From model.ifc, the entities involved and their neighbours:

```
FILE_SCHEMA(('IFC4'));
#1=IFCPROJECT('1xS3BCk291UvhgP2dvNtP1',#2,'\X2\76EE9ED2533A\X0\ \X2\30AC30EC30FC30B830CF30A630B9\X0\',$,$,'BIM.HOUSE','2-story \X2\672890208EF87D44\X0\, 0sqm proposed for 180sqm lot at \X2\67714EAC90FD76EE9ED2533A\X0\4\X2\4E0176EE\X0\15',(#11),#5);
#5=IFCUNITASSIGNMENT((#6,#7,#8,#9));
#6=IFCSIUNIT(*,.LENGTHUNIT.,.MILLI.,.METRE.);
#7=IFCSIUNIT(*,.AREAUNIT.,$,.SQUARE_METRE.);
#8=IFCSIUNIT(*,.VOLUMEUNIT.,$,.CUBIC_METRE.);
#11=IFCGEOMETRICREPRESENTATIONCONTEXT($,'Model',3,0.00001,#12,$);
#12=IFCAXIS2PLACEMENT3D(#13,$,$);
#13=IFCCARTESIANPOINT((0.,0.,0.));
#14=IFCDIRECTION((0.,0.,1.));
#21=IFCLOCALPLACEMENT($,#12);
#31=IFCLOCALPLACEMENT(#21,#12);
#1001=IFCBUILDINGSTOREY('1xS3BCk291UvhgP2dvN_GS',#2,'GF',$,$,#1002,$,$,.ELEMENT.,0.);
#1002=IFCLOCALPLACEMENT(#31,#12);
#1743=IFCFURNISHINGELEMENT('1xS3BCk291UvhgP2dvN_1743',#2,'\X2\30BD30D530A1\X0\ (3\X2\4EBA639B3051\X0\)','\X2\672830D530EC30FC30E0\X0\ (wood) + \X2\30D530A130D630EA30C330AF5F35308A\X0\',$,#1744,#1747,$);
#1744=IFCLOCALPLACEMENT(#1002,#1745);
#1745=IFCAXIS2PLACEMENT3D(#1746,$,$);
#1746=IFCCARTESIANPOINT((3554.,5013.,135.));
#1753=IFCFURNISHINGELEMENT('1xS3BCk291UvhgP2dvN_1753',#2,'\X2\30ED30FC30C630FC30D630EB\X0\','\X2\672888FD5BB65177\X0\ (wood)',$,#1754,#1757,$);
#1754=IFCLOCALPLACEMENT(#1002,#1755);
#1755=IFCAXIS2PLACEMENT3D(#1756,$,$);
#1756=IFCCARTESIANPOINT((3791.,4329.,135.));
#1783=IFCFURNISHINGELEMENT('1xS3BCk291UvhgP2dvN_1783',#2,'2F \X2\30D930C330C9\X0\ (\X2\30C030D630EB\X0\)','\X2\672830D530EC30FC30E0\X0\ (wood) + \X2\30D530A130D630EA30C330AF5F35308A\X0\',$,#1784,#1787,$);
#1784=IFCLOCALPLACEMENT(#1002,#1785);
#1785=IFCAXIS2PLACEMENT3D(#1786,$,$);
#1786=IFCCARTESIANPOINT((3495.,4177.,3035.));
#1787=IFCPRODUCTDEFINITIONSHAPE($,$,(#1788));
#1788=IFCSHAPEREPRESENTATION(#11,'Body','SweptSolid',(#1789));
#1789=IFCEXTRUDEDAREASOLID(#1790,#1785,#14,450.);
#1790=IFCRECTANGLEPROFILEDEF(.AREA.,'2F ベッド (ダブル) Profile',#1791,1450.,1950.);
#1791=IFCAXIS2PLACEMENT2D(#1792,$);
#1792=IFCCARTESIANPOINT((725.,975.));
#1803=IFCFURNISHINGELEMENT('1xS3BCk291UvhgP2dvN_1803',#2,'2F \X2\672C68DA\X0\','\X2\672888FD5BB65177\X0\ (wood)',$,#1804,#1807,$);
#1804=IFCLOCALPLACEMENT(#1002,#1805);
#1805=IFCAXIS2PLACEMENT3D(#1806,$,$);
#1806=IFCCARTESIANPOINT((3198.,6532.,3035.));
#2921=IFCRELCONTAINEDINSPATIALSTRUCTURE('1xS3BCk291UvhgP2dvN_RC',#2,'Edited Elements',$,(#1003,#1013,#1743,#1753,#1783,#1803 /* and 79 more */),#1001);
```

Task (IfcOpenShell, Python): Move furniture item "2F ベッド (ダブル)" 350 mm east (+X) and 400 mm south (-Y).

```python
import ifcopenshell
import ifcopenshell.api.geometry
import ifcopenshell.util.placement
import ifcopenshell.util.unit

model = ifcopenshell.open("model.ifc")
unit_scale = ifcopenshell.util.unit.calculate_unit_scale(model)

item = model.by_guid("1xS3BCk291UvhgP2dvN_1783")
matrix = ifcopenshell.util.placement.get_local_placement(item.ObjectPlacement)
matrix[0, 3] += 0.35 / unit_scale
matrix[1, 3] -= 0.4 / unit_scale
ifcopenshell.api.geometry.edit_object_placement(model, product=item, matrix=matrix, is_si=False)

print(ifcopenshell.util.placement.get_local_placement(item.ObjectPlacement).round(3) + 0.0)

model.write("model_rev.ifc")
```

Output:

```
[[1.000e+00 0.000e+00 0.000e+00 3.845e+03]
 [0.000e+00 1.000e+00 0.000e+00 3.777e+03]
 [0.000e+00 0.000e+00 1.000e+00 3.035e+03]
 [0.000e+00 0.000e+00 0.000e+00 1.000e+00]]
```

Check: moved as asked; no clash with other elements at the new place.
